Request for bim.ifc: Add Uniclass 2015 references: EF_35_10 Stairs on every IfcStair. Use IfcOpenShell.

First a look at what the model holds.

```python
import ifcopenshell

model = ifcopenshell.open("bim.ifc")
print(model.schema)
print("classifications:", [c.Name for c in model.by_type("IfcClassification")])
for ifc_class in ("IfcDoor", "IfcRoof", "IfcStair", "IfcWall", "IfcWindow"):
    print(ifc_class, len(model.by_type(ifc_class)))
```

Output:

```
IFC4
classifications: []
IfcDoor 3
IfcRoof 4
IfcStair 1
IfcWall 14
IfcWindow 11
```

```python
import ifcopenshell
import ifcopenshell.api.classification

model = ifcopenshell.open("bim.ifc")

system = ifcopenshell.api.classification.add_classification(model, classification="Uniclass 2015")

codes = {
    "IfcStair": ("EF_35_10", "Stairs"),
}
for ifc_class, (code, name) in codes.items():
    products = model.by_type(ifc_class)
    ifcopenshell.api.classification.add_reference(
        model, products=products, classification=system, identification=code, name=name
    )
    print(code, len(products))

model.write("bim_updated.ifc")
```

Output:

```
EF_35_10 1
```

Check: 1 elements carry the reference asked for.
